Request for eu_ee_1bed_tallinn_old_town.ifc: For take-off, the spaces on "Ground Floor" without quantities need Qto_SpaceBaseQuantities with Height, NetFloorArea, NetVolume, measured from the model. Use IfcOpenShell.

First a look at what the model holds.

```python
import ifcopenshell
import ifcopenshell.util.element
import ifcopenshell.util.unit

model = ifcopenshell.open("eu_ee_1bed_tallinn_old_town.ifc")
print(model.schema)
for unit_type in ("LENGTHUNIT", "AREAUNIT", "VOLUMEUNIT"):
    print(unit_type, ifcopenshell.util.unit.calculate_unit_scale(model, unit_type))
storey = next(s for s in model.by_type("IfcBuildingStorey") if s.Name == "Ground Floor")
spaces = [e for e in ifcopenshell.util.element.get_decomposition(storey) if e.is_a("IfcSpace")]
for e in sorted(spaces, key=lambda e: e.id()):
    print(e.id(), e.is_a(), e.Name, list(ifcopenshell.util.element.get_psets(e, qtos_only=True)), sep=" | ")
```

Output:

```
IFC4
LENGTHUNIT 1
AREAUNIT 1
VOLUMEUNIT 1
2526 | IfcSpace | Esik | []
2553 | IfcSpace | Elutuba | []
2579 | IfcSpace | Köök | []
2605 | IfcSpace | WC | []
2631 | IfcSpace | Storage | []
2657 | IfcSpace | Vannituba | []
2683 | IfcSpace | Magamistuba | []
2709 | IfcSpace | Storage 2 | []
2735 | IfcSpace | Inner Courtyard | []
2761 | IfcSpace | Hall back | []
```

```python
import ifcopenshell
import ifcopenshell.api.pset
import ifcopenshell.geom
import ifcopenshell.util.element
import ifcopenshell.util.shape
import ifcopenshell.util.unit

model = ifcopenshell.open("eu_ee_1bed_tallinn_old_town.ifc")
unit_scale = ifcopenshell.util.unit.calculate_unit_scale(model)
area_scale = ifcopenshell.util.unit.calculate_unit_scale(model, "AREAUNIT")
volume_scale = ifcopenshell.util.unit.calculate_unit_scale(model, "VOLUMEUNIT")
settings = ifcopenshell.geom.settings()

storey = next(s for s in model.by_type("IfcBuildingStorey") if s.Name == "Ground Floor")
spaces = [e for e in ifcopenshell.util.element.get_decomposition(storey) if e.is_a("IfcSpace")]

for e in sorted(spaces, key=lambda e: e.id()):
    if ifcopenshell.util.element.get_psets(e, qtos_only=True, should_inherit=False):
        continue
    # Geometry comes back in metres, in the element's own axes.
    shape = ifcopenshell.geom.create_shape(settings, e)
    values = {
        "Height": ifcopenshell.util.shape.get_z(shape.geometry) / unit_scale,
        "NetFloorArea": ifcopenshell.util.shape.get_footprint_area(shape.geometry) / area_scale,
        "NetVolume": ifcopenshell.util.shape.get_volume(shape.geometry) / volume_scale,
    }
    qto = ifcopenshell.api.pset.add_qto(model, product=e, name="Qto_SpaceBaseQuantities")
    ifcopenshell.api.pset.edit_qto(model, qto=qto, properties=values)
    print(e.id(), {k: round(v, 3) for k, v in values.items()})

model.write("eu_ee_1bed_tallinn_old_town-out.ifc")
```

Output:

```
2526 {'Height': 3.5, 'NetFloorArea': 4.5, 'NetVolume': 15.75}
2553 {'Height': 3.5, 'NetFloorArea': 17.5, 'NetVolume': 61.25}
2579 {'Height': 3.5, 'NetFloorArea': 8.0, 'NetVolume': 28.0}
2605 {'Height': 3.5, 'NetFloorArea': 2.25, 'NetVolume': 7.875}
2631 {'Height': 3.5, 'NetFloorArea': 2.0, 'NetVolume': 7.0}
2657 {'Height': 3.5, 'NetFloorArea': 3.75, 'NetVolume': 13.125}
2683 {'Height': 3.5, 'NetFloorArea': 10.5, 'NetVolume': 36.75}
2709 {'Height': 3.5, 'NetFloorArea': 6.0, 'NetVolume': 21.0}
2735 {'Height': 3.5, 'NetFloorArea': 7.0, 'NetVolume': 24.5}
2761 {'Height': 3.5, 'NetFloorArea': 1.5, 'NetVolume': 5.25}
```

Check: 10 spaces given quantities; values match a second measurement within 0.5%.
